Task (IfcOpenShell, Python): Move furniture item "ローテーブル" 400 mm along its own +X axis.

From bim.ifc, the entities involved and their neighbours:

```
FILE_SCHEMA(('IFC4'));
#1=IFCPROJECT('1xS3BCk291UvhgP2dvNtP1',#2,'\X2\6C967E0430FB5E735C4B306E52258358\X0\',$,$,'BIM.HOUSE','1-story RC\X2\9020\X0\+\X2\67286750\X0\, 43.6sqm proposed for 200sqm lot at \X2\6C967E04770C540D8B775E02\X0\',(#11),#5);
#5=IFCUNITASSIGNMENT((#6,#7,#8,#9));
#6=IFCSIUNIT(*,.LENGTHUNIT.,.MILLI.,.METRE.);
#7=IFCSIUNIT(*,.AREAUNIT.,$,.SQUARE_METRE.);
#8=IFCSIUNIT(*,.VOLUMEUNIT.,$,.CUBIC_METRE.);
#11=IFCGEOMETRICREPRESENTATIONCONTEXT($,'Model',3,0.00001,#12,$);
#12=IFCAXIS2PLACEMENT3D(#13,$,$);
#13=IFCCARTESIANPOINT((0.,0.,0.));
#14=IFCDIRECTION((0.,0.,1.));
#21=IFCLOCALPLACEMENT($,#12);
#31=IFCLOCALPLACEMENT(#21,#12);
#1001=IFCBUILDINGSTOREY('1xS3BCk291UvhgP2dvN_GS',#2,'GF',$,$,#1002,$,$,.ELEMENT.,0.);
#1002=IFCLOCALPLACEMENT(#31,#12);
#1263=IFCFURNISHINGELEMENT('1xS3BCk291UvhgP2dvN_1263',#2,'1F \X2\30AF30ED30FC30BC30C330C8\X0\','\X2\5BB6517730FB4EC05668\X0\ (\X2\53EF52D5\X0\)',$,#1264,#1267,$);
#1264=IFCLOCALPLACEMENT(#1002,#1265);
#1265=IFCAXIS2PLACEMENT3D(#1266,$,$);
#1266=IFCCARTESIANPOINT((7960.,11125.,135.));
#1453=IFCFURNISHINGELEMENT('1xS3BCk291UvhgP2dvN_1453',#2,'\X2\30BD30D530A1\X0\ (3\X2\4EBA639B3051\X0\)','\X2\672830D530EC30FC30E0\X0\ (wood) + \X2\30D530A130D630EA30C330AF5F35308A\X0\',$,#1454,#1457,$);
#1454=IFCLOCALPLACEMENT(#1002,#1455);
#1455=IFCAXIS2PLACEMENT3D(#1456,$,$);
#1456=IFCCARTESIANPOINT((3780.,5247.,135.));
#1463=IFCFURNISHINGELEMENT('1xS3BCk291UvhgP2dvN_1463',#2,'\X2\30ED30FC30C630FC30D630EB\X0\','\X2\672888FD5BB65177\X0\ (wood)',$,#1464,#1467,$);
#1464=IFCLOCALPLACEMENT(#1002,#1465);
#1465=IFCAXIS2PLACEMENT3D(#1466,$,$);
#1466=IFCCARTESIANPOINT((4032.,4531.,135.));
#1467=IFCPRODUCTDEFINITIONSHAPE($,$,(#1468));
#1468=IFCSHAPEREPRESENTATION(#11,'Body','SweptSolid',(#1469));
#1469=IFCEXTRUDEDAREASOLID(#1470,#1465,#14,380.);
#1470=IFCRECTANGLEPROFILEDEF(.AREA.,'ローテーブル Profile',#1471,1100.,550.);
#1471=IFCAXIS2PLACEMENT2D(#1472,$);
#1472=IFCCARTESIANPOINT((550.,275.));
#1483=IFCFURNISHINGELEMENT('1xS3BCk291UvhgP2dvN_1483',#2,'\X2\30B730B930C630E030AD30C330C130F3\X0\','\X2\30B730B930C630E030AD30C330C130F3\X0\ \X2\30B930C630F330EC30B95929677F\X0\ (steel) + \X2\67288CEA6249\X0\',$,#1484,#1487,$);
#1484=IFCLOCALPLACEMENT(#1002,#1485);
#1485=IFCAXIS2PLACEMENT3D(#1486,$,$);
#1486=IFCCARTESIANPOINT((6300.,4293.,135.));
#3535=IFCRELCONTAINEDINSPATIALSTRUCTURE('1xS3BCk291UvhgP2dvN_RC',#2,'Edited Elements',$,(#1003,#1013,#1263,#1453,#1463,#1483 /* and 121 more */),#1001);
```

```python
import ifcopenshell
import ifcopenshell.api.geometry
import ifcopenshell.util.placement
import ifcopenshell.util.unit

model = ifcopenshell.open("bim.ifc")
unit_scale = ifcopenshell.util.unit.calculate_unit_scale(model)

item = model.by_guid("1xS3BCk291UvhgP2dvN_1463")
matrix = ifcopenshell.util.placement.get_local_placement(item.ObjectPlacement)
matrix[:3, 3] += matrix[:3, 0] * 0.4 / unit_scale
ifcopenshell.api.geometry.edit_object_placement(model, product=item, matrix=matrix, is_si=False)

print(ifcopenshell.util.placement.get_local_placement(item.ObjectPlacement).round(3) + 0.0)

model.write("bim_updated.ifc")
```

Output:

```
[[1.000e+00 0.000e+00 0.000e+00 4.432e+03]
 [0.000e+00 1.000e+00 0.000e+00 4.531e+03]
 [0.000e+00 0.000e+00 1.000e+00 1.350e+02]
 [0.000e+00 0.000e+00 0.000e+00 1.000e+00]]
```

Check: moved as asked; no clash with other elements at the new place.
